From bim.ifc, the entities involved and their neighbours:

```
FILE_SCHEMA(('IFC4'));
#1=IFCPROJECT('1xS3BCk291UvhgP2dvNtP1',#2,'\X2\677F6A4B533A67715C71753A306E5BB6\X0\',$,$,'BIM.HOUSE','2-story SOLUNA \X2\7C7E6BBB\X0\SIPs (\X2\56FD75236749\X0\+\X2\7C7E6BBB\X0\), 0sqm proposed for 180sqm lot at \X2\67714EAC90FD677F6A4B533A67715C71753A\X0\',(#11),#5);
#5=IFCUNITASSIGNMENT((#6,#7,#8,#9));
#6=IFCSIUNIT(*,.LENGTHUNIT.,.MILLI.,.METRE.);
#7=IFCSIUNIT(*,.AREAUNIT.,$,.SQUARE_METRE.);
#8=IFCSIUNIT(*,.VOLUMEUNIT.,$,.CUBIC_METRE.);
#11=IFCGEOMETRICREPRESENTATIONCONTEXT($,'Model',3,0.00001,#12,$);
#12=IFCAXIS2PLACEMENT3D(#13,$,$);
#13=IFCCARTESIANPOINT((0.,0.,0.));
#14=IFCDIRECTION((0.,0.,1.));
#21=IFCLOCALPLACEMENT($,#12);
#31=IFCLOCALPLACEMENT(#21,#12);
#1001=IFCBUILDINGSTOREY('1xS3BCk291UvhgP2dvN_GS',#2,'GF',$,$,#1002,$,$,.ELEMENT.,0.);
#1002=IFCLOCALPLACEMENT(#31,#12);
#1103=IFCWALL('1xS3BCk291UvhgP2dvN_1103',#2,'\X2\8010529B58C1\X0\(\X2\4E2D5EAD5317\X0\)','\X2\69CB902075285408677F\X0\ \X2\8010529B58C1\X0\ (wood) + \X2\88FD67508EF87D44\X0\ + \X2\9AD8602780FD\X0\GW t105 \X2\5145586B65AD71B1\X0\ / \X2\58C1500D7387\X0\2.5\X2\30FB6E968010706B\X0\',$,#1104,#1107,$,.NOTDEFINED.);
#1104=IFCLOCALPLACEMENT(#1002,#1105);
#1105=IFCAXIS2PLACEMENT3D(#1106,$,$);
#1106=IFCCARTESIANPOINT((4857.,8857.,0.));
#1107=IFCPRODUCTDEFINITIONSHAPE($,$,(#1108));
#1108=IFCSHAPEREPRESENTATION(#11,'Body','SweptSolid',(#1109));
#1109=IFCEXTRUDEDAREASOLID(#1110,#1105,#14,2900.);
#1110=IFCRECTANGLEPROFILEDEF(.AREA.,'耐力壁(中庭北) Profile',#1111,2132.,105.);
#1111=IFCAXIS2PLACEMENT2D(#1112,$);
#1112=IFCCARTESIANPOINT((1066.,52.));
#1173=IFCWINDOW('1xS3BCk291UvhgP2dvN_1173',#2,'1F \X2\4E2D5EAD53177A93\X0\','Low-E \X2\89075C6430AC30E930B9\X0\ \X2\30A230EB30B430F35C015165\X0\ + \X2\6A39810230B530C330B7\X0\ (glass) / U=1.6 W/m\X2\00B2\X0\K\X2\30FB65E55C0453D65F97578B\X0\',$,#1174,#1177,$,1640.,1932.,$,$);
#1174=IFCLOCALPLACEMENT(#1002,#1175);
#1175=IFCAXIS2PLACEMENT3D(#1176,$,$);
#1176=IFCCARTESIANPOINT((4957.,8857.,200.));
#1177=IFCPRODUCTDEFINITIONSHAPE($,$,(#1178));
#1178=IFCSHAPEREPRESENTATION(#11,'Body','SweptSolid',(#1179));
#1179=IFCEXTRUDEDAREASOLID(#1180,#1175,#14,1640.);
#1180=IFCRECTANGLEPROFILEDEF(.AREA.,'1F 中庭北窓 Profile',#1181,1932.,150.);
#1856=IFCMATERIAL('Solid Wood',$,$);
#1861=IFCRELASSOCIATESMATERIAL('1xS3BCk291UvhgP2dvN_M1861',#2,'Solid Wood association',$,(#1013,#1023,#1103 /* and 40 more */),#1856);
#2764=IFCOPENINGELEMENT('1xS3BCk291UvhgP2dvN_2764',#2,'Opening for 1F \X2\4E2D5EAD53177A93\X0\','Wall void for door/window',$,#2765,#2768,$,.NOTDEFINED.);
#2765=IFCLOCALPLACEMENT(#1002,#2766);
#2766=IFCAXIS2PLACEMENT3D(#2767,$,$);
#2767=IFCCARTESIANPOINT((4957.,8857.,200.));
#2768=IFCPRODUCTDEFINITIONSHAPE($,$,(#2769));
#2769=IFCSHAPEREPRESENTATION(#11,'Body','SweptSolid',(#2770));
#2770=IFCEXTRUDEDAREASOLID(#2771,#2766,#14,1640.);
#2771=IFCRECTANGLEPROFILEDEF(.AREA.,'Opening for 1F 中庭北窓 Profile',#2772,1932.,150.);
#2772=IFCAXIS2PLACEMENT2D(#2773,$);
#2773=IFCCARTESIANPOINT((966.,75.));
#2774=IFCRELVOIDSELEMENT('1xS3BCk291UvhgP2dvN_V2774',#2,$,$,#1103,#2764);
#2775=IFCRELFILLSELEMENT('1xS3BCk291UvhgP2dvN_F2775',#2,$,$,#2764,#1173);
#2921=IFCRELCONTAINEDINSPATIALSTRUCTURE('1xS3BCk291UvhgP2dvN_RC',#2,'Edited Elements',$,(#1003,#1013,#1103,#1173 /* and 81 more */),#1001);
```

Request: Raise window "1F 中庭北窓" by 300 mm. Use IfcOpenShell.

```python
import numpy as np
import ifcopenshell
import ifcopenshell.api.geometry
import ifcopenshell.util.placement
import ifcopenshell.util.unit

model = ifcopenshell.open("bim.ifc")
unit_scale = ifcopenshell.util.unit.calculate_unit_scale(model)

window = model.by_guid("1xS3BCk291UvhgP2dvN_1173")
opening = window.FillsVoids[0].RelatingOpeningElement
dz = 300.0

shift = np.array([0.0, 0.0, dz])
# The window is not placed relative to its opening, so move both.
for product in (opening, window):
    matrix = ifcopenshell.util.placement.get_local_placement(product.ObjectPlacement)
    matrix[:3, 3] += shift
    ifcopenshell.api.geometry.edit_object_placement(model, product=product, matrix=matrix, is_si=False)

print(f"moved by {dz * unit_scale:+.3f} m")

model.write("bim_updated.ifc")
```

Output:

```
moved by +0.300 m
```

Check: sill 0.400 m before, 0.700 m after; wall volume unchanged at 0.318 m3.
